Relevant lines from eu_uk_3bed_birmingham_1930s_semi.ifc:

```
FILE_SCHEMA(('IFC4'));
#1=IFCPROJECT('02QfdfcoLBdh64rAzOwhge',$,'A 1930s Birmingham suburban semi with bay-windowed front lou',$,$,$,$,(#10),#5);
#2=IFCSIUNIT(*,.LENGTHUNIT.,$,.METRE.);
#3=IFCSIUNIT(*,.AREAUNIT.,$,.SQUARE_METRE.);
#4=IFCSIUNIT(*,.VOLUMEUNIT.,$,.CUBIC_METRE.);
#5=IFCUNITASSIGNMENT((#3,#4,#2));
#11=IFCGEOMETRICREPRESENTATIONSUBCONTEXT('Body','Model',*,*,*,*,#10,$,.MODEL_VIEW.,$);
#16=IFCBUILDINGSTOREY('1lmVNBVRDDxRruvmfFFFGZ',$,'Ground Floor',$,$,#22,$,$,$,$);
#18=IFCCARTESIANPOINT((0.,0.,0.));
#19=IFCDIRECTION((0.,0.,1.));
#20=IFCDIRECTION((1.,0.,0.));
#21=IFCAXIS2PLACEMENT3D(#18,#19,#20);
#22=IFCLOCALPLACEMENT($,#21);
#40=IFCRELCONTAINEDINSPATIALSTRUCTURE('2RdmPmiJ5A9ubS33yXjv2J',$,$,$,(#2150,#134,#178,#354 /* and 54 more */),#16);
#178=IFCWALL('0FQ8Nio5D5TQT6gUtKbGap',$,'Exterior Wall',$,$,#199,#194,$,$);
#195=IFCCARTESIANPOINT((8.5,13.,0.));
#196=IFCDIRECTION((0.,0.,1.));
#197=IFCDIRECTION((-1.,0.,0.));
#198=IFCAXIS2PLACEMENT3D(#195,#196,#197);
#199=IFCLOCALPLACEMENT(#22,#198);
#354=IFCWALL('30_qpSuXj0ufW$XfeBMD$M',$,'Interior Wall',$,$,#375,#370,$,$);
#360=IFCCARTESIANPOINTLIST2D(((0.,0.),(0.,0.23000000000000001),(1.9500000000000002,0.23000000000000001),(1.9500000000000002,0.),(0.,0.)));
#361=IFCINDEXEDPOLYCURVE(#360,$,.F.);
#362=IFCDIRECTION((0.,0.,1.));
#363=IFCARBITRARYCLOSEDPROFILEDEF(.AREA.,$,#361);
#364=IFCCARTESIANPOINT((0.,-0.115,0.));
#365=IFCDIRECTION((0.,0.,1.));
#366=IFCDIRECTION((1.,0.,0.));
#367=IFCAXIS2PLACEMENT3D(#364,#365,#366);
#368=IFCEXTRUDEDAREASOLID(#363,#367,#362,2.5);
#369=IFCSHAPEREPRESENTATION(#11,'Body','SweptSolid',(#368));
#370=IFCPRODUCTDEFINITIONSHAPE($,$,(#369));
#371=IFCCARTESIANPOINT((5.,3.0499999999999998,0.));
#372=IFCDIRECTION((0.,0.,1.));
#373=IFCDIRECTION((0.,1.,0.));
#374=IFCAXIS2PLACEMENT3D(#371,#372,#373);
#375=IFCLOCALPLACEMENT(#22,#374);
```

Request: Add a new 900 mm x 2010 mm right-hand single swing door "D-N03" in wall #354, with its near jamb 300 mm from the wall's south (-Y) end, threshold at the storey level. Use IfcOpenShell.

```python
import numpy as np
import ifcopenshell
import ifcopenshell.api.feature
import ifcopenshell.api.geometry
import ifcopenshell.api.root
import ifcopenshell.api.spatial
import ifcopenshell.geom
import ifcopenshell.util.element
import ifcopenshell.util.placement
import ifcopenshell.util.representation
import ifcopenshell.util.shape
import ifcopenshell.util.unit

model = ifcopenshell.open("eu_uk_3bed_birmingham_1930s_semi.ifc")
unit_scale = ifcopenshell.util.unit.calculate_unit_scale(model)
settings = ifcopenshell.geom.settings()


def volume(element):
    """Net volume in cubic metres, openings subtracted."""
    shape = ifcopenshell.geom.create_shape(settings, element)
    return ifcopenshell.util.shape.get_volume(shape.geometry)


wall = model.by_guid("30_qpSuXj0ufW$XfeBMD$M")
storey = ifcopenshell.util.element.get_container(wall, ifc_class="IfcBuildingStorey")
context = ifcopenshell.util.representation.get_context(model, "Model", "Body", "MODEL_VIEW")
before = volume(wall)

width, height, from_end, sill = 0.9, 2.01, 0.3, 0.0  # metres

# The wall runs along its own X axis, and the end named is its -X end.
wall_shape = ifcopenshell.geom.create_shape(settings, wall)
x, y, z = ifcopenshell.util.shape.get_vertices(wall_shape.geometry).T
start = x.min() + from_end
face, thickness = float(y.min()), float(y.max() - y.min())
wall_matrix = ifcopenshell.util.placement.get_local_placement(wall.ObjectPlacement)
level = ifcopenshell.util.placement.get_local_placement(storey.ObjectPlacement)[2, 3]


def in_wall(x, y):
    """Placement at x, y metres in the wall's axes, at sill height."""
    matrix = wall_matrix.copy()
    matrix[:, 3] = wall_matrix @ np.array([x / unit_scale, y / unit_scale, 0.0, 1.0])
    matrix[2, 3] = level + sill / unit_scale
    return matrix


# Opening: a box that overshoots both wall faces by 50 mm.
opening = ifcopenshell.api.root.create_entity(model, ifc_class="IfcOpeningElement", predefined_type="OPENING")
box = ifcopenshell.api.geometry.add_wall_representation(
    model, context=context, length=width, height=height, thickness=thickness + 0.1
)
ifcopenshell.api.geometry.assign_representation(model, product=opening, representation=box)
ifcopenshell.api.geometry.edit_object_placement(model, product=opening, matrix=in_wall(start, face - 0.05), is_si=False)
ifcopenshell.api.feature.add_feature(model, feature=opening, element=wall)

door = ifcopenshell.api.root.create_entity(model, ifc_class="IfcDoor", name="D-N03", predefined_type="DOOR")
door.OverallWidth, door.OverallHeight = width / unit_scale, height / unit_scale
door.OperationType = "SINGLE_SWING_RIGHT"
body = ifcopenshell.api.geometry.add_door_representation(
    model,
    context=context,
    overall_width=door.OverallWidth,
    overall_height=door.OverallHeight,
    operation_type="SINGLE_SWING_RIGHT",
    lining_properties={"LiningDepth": thickness / unit_scale, "ThresholdDepth": thickness / unit_scale},
)
ifcopenshell.api.geometry.assign_representation(model, product=door, representation=body)
ifcopenshell.api.spatial.assign_container(model, products=[door], relating_structure=storey)
ifcopenshell.api.feature.add_filling(model, opening=opening, element=door)

# The lining spans the wall, so the door starts at the wall face.
ifcopenshell.api.geometry.edit_object_placement(model, product=door, matrix=in_wall(start, face), is_si=False)

after = volume(wall)

print(f"wall volume {before:.3f} -> {after:.3f} m3")

model.write("eu_uk_3bed_birmingham_1930s_semi_edited.ifc")
```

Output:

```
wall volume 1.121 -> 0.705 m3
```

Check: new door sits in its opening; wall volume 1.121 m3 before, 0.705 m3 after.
